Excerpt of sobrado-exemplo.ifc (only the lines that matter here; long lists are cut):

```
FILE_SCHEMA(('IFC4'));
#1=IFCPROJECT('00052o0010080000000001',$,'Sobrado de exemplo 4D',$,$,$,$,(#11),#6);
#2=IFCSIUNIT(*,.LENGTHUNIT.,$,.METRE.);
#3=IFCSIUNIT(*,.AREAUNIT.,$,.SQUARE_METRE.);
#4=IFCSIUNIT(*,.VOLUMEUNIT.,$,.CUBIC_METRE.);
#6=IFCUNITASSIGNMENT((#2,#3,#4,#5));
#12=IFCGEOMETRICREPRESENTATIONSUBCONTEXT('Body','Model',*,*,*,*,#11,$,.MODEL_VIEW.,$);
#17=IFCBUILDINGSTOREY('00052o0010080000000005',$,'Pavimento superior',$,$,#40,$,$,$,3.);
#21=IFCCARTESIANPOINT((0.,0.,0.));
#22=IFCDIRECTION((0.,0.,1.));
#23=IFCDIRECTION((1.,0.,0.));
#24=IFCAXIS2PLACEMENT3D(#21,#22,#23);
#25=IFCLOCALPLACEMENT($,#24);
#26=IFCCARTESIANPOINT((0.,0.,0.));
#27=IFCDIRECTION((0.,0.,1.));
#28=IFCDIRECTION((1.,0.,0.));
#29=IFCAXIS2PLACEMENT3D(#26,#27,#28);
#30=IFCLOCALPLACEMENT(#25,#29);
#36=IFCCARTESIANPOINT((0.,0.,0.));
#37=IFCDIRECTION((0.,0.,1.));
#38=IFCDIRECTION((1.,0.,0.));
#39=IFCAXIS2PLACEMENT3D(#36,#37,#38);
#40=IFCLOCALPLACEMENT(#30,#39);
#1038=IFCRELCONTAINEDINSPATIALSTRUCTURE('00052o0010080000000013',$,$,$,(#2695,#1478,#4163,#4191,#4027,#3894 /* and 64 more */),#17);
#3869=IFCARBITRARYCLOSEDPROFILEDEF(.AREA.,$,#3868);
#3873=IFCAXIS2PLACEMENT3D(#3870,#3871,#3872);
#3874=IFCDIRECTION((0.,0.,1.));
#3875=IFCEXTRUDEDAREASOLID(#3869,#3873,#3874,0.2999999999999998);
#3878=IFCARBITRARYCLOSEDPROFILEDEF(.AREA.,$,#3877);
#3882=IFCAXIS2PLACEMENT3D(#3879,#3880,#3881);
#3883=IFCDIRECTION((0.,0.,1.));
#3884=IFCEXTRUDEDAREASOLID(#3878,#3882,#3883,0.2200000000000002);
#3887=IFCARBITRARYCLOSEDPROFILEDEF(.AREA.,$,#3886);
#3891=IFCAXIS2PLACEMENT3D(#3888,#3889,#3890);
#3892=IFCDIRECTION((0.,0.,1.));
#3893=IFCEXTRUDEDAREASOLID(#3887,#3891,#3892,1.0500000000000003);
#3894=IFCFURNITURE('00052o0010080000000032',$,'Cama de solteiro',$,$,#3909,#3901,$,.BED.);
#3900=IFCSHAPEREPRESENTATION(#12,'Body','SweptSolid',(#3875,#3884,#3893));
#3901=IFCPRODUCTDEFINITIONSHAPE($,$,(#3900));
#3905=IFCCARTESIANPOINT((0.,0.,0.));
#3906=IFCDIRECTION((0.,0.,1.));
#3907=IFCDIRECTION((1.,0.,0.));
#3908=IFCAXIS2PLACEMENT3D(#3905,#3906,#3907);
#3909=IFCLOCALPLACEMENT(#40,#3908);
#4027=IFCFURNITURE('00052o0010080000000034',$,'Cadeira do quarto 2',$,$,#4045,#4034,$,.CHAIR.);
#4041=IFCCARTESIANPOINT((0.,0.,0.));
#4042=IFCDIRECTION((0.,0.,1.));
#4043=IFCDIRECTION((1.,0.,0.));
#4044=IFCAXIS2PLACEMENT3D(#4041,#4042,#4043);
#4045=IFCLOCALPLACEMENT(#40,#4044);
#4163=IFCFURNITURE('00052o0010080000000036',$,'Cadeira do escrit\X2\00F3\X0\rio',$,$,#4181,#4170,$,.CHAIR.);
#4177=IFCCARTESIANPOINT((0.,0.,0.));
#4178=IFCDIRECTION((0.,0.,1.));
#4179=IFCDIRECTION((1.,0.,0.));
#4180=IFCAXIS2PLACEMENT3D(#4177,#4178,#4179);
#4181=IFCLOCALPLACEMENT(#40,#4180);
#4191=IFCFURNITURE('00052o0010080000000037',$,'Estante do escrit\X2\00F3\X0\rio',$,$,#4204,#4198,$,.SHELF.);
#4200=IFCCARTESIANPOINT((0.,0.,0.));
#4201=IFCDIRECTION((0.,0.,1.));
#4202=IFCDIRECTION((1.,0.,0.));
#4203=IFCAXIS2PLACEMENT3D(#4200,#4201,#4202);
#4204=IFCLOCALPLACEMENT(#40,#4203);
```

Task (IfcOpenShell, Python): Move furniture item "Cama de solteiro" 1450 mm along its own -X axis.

```python
import ifcopenshell
import ifcopenshell.api.geometry
import ifcopenshell.util.placement
import ifcopenshell.util.unit

model = ifcopenshell.open("sobrado-exemplo.ifc")
unit_scale = ifcopenshell.util.unit.calculate_unit_scale(model)

item = model.by_guid("00052o0010080000000032")
matrix = ifcopenshell.util.placement.get_local_placement(item.ObjectPlacement)
matrix[:3, 3] -= matrix[:3, 0] * 1.45 / unit_scale
ifcopenshell.api.geometry.edit_object_placement(model, product=item, matrix=matrix, is_si=False)

print(ifcopenshell.util.placement.get_local_placement(item.ObjectPlacement).round(3) + 0.0)

model.write("sobrado-exemplo_rev.ifc")
```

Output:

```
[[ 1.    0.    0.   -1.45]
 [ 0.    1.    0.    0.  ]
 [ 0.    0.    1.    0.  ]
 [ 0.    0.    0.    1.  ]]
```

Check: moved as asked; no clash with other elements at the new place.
